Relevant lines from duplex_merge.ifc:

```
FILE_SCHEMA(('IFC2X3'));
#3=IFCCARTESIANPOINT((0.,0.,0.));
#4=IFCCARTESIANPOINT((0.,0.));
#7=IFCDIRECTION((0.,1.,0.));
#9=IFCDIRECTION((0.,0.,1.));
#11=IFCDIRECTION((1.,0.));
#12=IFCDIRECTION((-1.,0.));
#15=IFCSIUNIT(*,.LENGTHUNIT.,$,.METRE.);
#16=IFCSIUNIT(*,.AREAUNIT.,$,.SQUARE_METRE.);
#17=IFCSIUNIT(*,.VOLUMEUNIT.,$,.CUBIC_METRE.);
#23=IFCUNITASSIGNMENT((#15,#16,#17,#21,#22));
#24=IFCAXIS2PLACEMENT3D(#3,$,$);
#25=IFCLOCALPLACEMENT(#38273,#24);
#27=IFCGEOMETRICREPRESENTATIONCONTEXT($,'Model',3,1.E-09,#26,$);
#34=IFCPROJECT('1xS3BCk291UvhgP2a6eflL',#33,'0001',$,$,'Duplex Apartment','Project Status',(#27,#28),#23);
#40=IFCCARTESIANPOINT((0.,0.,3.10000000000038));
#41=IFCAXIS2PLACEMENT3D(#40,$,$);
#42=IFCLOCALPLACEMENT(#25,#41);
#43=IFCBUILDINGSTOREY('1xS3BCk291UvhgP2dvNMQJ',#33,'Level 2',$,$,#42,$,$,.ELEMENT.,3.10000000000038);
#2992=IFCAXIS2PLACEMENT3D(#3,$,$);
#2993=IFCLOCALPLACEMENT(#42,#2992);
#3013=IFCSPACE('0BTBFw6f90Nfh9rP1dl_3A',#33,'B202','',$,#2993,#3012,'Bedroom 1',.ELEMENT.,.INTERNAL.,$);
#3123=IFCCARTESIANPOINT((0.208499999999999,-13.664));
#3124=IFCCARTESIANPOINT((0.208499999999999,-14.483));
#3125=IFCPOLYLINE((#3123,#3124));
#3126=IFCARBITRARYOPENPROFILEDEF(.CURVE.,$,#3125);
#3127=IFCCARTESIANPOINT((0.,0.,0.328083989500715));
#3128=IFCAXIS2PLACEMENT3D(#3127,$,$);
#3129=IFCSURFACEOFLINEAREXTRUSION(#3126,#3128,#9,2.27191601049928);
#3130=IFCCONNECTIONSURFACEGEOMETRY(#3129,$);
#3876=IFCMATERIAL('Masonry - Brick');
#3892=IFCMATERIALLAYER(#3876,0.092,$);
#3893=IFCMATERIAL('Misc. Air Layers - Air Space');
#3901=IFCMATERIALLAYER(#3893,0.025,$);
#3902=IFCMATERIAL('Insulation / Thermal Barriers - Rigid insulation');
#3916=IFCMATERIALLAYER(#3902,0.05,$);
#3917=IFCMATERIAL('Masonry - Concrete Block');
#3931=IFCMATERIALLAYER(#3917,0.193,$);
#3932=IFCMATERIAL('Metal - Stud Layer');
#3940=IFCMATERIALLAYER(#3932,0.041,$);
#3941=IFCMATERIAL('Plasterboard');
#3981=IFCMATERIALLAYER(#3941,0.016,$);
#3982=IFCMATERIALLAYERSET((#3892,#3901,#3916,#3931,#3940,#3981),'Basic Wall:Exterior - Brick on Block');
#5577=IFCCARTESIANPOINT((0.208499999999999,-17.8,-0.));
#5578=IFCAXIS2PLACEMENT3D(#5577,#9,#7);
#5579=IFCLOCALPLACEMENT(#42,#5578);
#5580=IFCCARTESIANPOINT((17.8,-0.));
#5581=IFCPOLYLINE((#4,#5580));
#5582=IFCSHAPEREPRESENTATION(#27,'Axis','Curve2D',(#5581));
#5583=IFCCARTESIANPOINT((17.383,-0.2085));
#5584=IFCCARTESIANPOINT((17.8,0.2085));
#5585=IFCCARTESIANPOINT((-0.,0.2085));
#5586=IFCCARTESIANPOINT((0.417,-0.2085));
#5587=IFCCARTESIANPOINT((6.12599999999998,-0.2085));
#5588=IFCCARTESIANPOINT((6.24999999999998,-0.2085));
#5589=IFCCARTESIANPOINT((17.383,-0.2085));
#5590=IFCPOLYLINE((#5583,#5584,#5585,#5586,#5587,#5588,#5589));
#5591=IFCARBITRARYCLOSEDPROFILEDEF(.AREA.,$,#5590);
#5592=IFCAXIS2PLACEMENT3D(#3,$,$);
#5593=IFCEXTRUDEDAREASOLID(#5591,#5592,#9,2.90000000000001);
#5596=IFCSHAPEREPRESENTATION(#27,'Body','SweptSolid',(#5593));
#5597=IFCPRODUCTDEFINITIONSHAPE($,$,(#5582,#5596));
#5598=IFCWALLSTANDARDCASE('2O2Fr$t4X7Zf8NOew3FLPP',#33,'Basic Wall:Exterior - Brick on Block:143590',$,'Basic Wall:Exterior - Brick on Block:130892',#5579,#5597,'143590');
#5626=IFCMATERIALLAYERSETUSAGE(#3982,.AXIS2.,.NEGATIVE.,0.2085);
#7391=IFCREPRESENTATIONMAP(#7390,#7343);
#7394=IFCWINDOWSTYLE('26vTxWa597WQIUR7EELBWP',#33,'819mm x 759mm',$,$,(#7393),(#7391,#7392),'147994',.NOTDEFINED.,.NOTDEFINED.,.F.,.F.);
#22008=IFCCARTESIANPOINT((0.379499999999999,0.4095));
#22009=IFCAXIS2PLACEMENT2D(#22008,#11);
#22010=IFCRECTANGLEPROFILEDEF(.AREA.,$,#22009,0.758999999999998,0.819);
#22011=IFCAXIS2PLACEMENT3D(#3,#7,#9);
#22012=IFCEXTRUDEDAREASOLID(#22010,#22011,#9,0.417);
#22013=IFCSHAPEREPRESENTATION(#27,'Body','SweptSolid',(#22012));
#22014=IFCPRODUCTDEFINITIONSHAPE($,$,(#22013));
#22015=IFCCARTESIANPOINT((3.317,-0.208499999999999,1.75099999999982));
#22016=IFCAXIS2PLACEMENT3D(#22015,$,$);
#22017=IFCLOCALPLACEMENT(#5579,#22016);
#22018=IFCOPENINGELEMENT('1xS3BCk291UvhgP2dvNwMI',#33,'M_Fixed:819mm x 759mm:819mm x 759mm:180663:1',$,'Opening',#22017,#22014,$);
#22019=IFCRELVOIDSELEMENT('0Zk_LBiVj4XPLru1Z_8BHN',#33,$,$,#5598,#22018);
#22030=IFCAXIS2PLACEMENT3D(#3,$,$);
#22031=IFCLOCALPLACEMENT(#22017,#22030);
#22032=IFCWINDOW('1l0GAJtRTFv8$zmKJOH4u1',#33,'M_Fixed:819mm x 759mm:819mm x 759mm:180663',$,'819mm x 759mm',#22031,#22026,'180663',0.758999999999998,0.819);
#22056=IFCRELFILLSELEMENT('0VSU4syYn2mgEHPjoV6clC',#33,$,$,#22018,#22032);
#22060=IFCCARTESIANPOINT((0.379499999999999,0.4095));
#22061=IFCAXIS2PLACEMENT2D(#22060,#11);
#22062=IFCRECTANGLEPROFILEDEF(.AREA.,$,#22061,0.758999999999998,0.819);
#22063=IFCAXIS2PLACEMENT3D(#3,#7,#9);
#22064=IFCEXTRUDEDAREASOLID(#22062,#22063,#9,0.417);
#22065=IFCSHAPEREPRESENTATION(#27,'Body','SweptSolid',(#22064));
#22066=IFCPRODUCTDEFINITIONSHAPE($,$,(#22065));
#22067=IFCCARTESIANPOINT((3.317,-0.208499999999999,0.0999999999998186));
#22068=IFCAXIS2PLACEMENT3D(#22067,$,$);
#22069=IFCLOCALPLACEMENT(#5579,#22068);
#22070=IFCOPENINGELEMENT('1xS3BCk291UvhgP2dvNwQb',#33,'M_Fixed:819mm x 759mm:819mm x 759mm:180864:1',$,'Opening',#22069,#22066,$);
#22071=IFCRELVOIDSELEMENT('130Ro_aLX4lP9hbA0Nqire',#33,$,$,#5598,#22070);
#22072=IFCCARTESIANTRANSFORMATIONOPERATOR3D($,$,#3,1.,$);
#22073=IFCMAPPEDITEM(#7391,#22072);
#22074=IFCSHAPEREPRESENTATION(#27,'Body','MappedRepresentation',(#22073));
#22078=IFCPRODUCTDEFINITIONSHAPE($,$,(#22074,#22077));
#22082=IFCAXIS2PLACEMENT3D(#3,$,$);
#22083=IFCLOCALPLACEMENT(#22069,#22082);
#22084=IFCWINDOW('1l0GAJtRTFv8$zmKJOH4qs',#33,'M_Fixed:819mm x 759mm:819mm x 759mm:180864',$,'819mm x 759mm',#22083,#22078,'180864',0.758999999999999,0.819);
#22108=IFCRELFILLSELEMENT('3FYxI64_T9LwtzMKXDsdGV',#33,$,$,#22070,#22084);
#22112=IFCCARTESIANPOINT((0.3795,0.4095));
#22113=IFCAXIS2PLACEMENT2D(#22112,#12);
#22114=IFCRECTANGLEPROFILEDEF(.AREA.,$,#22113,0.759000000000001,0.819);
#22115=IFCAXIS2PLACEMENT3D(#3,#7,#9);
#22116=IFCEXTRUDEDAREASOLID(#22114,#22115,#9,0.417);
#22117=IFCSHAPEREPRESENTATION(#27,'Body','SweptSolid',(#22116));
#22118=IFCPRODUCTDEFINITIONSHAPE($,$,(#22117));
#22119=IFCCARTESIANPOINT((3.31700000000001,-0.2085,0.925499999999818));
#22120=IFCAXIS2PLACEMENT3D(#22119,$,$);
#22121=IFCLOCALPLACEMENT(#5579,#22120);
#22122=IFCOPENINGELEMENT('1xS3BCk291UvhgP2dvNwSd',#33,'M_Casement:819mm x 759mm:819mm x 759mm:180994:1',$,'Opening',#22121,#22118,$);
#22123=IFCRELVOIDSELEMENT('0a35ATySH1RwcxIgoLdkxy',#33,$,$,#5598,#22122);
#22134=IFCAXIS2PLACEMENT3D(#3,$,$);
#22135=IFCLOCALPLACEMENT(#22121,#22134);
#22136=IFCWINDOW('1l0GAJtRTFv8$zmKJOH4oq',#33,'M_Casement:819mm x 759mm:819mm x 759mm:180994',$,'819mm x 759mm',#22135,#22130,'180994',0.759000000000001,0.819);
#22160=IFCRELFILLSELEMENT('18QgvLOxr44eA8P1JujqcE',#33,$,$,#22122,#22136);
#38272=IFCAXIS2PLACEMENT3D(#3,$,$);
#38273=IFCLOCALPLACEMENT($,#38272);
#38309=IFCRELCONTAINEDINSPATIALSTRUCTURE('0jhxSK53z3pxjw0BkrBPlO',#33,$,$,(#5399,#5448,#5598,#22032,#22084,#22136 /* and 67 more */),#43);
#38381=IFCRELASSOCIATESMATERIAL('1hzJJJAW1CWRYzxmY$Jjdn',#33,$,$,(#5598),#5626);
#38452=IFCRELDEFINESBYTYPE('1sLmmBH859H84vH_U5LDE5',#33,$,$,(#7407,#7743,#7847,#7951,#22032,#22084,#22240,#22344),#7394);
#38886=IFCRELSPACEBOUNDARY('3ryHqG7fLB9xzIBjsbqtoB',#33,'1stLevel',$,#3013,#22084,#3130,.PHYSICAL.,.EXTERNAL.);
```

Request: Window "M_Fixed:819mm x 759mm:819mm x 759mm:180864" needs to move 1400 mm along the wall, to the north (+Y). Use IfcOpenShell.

```python
import numpy as np
import ifcopenshell
import ifcopenshell.api.geometry
import ifcopenshell.util.placement

model = ifcopenshell.open("duplex_merge.ifc")

window = model.by_guid("1l0GAJtRTFv8$zmKJOH4qs")
opening = window.FillsVoids[0].RelatingOpeningElement
wall = opening.VoidsElements[0].RelatingBuildingElement

wall_matrix = ifcopenshell.util.placement.get_local_placement(wall.ObjectPlacement)
shift = wall_matrix[:3, 0] * 1.4
before = ifcopenshell.util.placement.get_local_placement(window.ObjectPlacement)[:3, 3].copy()

# The window is placed relative to its opening, so it follows when the opening moves.
matrix = ifcopenshell.util.placement.get_local_placement(opening.ObjectPlacement)
matrix[:3, 3] += shift
ifcopenshell.api.geometry.edit_object_placement(
    model, product=opening, matrix=matrix, is_si=False, should_transform_children=True
)

# Space boundary surfaces are stored in each space's coordinates; move them too.
for rel in window.ProvidesBoundaries:
    if not rel.ConnectionGeometry:
        continue
    surface = rel.ConnectionGeometry.SurfaceOnRelatingElement
    space_matrix = ifcopenshell.util.placement.get_local_placement(rel.RelatingSpace.ObjectPlacement)
    point = np.array(surface.Position.Location.Coordinates) + space_matrix[:3, :3].T @ shift
    surface.Position = model.createIfcAxis2Placement3D(
        model.createIfcCartesianPoint(point.tolist()), surface.Position.Axis, surface.Position.RefDirection
    )

after = ifcopenshell.util.placement.get_local_placement(window.ObjectPlacement)[:3, 3]
print("window moved by", (after - before).round(3) + 0.0)

model.write("duplex_merge_updated.ifc")
```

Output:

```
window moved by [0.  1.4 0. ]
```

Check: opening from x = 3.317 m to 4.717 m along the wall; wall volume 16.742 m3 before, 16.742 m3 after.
